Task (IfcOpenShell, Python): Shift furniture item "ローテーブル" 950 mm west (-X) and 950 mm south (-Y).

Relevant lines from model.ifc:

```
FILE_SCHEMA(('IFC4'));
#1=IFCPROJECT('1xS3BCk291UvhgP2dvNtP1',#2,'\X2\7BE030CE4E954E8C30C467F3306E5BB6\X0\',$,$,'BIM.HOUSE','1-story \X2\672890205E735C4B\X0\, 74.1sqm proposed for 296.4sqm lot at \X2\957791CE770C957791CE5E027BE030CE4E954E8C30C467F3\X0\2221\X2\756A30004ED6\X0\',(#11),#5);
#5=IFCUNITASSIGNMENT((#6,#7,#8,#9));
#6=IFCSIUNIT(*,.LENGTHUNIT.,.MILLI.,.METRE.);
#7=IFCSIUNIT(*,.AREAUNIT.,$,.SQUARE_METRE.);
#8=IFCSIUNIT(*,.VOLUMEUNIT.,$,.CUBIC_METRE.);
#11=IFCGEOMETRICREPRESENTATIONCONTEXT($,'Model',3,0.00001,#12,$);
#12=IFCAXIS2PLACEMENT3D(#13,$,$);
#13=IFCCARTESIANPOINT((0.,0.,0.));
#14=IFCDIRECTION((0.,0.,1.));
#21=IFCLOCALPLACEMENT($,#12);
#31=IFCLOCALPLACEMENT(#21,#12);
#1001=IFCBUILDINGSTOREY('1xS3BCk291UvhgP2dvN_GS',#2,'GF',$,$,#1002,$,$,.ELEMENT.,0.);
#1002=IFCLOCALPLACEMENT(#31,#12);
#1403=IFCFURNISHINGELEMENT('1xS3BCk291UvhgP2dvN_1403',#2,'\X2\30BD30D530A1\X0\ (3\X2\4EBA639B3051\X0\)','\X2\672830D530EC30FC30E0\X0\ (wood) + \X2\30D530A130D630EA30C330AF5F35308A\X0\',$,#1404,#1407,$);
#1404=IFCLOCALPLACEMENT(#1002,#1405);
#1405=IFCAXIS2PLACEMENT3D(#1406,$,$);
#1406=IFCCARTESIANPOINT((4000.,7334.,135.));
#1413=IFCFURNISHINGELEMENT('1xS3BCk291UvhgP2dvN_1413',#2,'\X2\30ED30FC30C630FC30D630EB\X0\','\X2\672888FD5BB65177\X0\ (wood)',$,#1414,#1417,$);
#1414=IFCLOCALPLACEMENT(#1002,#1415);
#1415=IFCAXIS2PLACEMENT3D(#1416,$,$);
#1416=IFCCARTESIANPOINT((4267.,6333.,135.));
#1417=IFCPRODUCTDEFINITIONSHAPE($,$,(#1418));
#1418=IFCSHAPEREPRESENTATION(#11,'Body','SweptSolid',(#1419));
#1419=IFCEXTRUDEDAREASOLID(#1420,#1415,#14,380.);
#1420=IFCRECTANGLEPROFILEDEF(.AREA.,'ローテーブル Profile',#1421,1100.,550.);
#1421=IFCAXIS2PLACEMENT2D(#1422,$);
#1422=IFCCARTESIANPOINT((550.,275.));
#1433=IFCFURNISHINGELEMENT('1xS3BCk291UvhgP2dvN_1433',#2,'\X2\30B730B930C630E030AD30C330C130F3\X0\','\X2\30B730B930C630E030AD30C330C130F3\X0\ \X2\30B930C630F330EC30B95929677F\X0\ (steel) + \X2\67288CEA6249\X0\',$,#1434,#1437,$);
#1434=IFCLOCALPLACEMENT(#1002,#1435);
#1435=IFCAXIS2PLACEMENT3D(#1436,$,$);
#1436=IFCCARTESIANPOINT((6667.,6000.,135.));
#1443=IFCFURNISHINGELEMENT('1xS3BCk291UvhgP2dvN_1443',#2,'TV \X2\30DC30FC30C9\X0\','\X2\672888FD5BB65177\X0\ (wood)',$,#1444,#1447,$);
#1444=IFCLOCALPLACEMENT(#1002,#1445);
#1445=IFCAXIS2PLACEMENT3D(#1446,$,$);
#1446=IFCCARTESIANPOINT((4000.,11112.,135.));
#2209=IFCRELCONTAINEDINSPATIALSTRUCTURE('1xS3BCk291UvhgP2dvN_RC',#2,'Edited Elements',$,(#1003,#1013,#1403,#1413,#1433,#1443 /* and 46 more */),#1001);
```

```python
import ifcopenshell
import ifcopenshell.api.geometry
import ifcopenshell.util.placement
import ifcopenshell.util.unit

model = ifcopenshell.open("model.ifc")
unit_scale = ifcopenshell.util.unit.calculate_unit_scale(model)

item = model.by_id(1413)
matrix = ifcopenshell.util.placement.get_local_placement(item.ObjectPlacement)
matrix[0, 3] -= 0.95 / unit_scale
matrix[1, 3] -= 0.95 / unit_scale
ifcopenshell.api.geometry.edit_object_placement(model, product=item, matrix=matrix, is_si=False)

print(ifcopenshell.util.placement.get_local_placement(item.ObjectPlacement).round(3) + 0.0)

model.write("model_v2.ifc")
```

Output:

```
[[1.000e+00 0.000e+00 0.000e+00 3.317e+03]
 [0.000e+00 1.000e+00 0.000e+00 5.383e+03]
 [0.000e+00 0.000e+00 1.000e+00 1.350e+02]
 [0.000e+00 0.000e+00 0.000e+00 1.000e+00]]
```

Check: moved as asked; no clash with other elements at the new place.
